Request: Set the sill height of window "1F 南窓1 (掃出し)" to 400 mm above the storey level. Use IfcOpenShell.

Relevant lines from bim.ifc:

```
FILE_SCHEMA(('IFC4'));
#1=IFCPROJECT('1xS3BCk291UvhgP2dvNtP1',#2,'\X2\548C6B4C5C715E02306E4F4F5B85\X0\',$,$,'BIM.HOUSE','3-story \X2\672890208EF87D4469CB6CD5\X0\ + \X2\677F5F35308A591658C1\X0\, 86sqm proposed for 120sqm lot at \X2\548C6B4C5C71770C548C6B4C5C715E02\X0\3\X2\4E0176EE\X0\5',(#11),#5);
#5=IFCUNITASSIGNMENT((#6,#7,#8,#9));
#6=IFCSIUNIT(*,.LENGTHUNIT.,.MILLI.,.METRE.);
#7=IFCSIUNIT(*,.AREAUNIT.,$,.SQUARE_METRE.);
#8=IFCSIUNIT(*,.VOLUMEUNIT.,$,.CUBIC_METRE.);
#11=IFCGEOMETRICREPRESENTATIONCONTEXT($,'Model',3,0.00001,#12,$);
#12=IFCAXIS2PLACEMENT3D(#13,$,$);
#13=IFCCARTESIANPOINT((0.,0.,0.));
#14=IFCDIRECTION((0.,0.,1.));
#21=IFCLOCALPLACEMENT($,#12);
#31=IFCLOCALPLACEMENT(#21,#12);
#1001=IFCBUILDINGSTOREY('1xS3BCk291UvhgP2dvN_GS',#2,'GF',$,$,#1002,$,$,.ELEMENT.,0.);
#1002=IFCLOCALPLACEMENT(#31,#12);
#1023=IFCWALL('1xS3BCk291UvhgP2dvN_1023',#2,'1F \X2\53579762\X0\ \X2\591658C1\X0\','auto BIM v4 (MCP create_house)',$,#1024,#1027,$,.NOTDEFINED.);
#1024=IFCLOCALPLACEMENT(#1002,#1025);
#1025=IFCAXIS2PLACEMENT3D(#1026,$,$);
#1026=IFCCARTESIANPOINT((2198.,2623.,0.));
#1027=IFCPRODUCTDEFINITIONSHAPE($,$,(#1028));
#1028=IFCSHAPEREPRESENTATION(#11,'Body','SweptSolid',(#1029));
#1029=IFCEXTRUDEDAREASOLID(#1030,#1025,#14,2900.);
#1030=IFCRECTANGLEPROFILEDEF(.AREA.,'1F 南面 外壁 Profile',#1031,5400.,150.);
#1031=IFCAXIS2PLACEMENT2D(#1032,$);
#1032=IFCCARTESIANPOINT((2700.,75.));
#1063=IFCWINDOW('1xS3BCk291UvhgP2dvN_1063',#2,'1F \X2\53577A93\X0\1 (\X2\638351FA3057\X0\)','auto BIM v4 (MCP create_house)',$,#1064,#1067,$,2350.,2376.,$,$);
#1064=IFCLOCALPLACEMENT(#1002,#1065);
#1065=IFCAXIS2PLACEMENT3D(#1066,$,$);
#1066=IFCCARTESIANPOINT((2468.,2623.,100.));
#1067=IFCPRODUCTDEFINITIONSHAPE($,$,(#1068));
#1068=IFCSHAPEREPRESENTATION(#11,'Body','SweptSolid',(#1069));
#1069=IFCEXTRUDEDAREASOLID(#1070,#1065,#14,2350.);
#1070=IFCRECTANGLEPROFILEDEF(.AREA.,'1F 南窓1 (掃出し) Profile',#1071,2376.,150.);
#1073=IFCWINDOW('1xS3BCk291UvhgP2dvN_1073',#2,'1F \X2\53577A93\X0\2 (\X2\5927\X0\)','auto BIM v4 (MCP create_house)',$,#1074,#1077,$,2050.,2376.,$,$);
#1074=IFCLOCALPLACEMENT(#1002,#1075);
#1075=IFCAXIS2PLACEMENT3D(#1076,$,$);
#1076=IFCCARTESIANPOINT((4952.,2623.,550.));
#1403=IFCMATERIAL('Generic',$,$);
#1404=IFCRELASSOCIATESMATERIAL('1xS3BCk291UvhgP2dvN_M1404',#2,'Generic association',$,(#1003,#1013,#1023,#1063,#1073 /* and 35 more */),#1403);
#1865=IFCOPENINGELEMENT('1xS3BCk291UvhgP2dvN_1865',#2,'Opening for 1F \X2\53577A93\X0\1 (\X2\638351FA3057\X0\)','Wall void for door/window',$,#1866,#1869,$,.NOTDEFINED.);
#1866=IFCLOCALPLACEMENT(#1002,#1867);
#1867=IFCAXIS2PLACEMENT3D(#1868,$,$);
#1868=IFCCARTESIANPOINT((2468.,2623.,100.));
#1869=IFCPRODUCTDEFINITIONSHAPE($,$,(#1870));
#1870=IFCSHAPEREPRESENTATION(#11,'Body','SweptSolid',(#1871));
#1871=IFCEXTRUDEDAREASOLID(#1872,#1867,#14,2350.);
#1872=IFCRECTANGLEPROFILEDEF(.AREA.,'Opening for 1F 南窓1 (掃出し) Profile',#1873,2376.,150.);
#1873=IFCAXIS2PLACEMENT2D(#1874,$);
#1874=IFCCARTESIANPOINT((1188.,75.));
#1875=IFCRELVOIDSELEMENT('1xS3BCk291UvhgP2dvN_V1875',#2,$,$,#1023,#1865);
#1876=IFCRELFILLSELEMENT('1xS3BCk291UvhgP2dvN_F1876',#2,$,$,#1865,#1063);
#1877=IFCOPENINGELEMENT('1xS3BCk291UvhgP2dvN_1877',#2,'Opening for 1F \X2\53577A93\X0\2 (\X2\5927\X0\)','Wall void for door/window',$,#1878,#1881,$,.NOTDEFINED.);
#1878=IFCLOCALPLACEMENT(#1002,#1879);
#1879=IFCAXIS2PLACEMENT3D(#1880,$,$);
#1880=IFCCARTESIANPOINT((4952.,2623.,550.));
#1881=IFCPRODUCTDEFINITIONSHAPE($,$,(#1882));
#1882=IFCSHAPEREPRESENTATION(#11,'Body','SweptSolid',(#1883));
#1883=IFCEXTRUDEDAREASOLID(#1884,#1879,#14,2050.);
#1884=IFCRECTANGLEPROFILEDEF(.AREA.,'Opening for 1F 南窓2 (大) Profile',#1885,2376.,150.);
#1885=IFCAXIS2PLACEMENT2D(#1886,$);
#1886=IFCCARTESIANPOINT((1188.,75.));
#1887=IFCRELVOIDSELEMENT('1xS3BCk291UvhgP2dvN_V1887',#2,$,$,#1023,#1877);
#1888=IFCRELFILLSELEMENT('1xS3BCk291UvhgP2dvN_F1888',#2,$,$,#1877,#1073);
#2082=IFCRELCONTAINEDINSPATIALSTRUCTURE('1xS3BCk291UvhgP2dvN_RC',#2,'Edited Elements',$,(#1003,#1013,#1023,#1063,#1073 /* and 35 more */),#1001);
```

```python
import numpy as np
import ifcopenshell
import ifcopenshell.api.geometry
import ifcopenshell.geom
import ifcopenshell.util.element
import ifcopenshell.util.placement
import ifcopenshell.util.shape
import ifcopenshell.util.unit

model = ifcopenshell.open("bim.ifc")
unit_scale = ifcopenshell.util.unit.calculate_unit_scale(model)

window = model.by_guid("1xS3BCk291UvhgP2dvN_1063")
opening = window.FillsVoids[0].RelatingOpeningElement
storey = ifcopenshell.util.element.get_container(window, ifc_class="IfcBuildingStorey")
level = ifcopenshell.util.placement.get_local_placement(storey.ObjectPlacement)[2, 3]

# The opening's origin need not be at the sill, so measure its lowest point.
shape = ifcopenshell.geom.create_shape(ifcopenshell.geom.settings(), opening)
bottom = ifcopenshell.util.shape.get_shape_bottom_elevation(shape, shape.geometry) / unit_scale
dz = level + 400.0 - bottom

shift = np.array([0.0, 0.0, dz])
# The window is not placed relative to its opening, so move both.
for product in (opening, window):
    matrix = ifcopenshell.util.placement.get_local_placement(product.ObjectPlacement)
    matrix[:3, 3] += shift
    ifcopenshell.api.geometry.edit_object_placement(model, product=product, matrix=matrix, is_si=False)

print(f"moved by {dz * unit_scale:+.3f} m")

model.write("bim_updated.ifc")
```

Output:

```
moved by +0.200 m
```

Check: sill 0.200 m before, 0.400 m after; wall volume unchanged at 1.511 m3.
